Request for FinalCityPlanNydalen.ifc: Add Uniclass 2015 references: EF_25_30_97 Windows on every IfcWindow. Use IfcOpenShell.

First a look at what the model holds.

```python
import ifcopenshell

model = ifcopenshell.open("FinalCityPlanNydalen.ifc")
print(model.schema)
print("classifications:", [c.Name for c in model.by_type("IfcClassification")])
for ifc_class in ("IfcDoor", "IfcRoof", "IfcStair", "IfcWall", "IfcWindow"):
    print(ifc_class, len(model.by_type(ifc_class)))
```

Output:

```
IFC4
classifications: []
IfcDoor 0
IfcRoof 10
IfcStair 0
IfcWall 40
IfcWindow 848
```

```python
import ifcopenshell
import ifcopenshell.api.classification

model = ifcopenshell.open("FinalCityPlanNydalen.ifc")

system = ifcopenshell.api.classification.add_classification(model, classification="Uniclass 2015")

codes = {
    "IfcWindow": ("EF_25_30_97", "Windows"),
}
for ifc_class, (code, name) in codes.items():
    products = model.by_type(ifc_class)
    ifcopenshell.api.classification.add_reference(
        model, products=products, classification=system, identification=code, name=name
    )
    print(code, len(products))

model.write("FinalCityPlanNydalen_edited.ifc")
```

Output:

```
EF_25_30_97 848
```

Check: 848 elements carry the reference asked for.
